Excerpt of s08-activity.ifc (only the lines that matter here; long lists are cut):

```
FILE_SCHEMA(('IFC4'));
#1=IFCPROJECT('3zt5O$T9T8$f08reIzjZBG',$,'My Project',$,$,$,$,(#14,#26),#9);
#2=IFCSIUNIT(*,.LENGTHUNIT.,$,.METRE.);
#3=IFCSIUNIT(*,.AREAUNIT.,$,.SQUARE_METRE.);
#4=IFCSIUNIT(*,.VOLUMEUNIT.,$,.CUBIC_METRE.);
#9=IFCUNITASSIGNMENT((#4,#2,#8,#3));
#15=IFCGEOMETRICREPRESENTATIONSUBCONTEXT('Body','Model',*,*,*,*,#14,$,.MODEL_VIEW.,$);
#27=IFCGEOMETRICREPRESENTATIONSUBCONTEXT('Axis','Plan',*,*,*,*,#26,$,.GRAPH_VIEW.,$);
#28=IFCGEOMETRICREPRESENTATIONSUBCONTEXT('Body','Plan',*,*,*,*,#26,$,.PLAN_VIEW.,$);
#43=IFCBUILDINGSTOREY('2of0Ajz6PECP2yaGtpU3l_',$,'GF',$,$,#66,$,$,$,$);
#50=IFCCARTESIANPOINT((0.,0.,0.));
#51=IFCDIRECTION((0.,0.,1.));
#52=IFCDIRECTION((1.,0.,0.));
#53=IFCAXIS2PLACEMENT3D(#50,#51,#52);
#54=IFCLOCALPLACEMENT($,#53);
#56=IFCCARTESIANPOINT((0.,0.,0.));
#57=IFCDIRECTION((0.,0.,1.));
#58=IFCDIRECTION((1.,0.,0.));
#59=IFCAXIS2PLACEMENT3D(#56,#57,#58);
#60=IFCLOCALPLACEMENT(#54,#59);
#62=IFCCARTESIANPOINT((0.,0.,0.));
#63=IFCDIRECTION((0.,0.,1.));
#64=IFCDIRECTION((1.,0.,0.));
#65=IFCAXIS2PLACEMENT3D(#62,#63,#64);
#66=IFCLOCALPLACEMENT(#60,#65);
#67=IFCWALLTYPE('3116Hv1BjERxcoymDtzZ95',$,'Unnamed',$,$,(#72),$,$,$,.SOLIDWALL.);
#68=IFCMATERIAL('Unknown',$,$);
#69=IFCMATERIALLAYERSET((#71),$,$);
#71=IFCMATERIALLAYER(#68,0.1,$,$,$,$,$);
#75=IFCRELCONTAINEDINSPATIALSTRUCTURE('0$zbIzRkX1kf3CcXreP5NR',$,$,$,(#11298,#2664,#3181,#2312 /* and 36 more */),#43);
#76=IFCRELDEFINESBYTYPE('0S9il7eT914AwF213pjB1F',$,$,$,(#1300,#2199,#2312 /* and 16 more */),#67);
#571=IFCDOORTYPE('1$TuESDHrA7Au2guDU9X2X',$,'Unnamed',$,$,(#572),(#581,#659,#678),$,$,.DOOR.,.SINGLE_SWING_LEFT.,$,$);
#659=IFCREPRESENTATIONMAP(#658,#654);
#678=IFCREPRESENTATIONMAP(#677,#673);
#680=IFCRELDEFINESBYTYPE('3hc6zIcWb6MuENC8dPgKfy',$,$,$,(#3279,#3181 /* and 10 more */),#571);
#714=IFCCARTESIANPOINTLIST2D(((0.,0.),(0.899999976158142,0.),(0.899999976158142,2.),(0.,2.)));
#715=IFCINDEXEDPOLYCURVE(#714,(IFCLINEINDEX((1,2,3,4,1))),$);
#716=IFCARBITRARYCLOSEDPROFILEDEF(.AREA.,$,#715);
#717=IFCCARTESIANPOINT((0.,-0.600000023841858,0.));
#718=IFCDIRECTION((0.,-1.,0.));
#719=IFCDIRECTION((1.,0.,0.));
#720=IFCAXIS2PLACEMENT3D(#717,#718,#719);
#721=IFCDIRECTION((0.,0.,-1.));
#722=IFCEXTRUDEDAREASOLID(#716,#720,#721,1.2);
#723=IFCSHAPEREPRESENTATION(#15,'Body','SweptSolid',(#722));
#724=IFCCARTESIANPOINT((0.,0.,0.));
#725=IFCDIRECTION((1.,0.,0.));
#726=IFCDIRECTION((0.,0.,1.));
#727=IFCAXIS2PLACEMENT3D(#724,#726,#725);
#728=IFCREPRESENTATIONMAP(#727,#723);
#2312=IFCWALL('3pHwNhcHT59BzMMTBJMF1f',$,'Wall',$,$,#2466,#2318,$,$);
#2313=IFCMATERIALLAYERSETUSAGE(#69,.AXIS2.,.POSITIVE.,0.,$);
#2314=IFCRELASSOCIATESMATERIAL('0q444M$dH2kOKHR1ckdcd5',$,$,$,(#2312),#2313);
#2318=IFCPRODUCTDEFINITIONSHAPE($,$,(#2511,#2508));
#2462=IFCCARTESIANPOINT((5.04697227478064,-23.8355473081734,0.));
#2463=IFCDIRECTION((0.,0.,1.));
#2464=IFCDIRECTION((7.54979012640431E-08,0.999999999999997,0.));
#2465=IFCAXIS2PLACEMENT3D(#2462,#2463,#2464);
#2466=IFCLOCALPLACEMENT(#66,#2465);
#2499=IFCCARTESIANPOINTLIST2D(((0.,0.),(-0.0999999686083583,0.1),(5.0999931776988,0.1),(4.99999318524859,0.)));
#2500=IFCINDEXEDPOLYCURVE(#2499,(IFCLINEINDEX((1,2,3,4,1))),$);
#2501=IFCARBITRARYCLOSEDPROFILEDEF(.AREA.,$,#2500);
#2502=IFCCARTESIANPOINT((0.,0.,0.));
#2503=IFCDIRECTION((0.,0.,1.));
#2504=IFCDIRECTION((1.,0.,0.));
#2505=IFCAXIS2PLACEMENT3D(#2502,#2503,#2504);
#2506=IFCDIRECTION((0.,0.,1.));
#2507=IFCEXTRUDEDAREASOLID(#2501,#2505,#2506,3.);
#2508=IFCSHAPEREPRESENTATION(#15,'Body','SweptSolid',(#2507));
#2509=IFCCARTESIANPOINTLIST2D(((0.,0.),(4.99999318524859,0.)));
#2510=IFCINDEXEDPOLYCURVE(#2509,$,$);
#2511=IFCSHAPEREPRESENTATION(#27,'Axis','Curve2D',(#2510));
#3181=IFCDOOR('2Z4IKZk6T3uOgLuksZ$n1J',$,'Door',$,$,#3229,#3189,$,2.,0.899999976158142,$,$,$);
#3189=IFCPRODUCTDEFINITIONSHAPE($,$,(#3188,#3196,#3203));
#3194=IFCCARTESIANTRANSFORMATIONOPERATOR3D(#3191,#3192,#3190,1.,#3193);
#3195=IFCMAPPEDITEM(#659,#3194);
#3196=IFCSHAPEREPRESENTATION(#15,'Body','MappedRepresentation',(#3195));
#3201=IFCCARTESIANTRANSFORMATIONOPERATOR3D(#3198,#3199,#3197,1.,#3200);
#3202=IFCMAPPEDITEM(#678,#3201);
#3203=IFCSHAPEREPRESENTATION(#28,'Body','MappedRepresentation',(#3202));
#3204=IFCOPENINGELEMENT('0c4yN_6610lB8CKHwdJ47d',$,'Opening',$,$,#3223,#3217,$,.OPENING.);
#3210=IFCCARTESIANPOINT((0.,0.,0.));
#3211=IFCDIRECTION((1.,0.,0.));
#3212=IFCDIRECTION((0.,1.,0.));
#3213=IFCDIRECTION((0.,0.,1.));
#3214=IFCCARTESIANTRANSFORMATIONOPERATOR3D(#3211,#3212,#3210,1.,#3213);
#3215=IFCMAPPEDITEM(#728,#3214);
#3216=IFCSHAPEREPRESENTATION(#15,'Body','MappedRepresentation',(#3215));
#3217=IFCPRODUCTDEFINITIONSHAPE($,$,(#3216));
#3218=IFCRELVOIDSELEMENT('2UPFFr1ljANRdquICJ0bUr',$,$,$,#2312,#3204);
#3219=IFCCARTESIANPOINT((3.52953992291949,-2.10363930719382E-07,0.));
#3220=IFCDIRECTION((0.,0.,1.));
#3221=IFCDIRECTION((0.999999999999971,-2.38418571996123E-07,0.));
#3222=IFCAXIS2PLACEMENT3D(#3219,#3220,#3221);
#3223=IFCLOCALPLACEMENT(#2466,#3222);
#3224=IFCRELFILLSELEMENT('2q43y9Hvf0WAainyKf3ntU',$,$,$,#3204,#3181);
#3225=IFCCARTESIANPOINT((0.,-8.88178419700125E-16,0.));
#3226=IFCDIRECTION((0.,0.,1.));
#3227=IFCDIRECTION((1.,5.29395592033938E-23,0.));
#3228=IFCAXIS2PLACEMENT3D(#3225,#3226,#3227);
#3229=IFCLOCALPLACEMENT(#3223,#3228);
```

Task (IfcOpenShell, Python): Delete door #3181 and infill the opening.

```python
import ifcopenshell
import ifcopenshell.api.feature
import ifcopenshell.api.root
import ifcopenshell.geom
import ifcopenshell.util.shape

model = ifcopenshell.open("s08-activity.ifc")
settings = ifcopenshell.geom.settings()


def volume(element):
    """Net volume in cubic metres, openings subtracted."""
    shape = ifcopenshell.geom.create_shape(settings, element)
    return ifcopenshell.util.shape.get_volume(shape.geometry)


door = model.by_id(3181)
opening = door.FillsVoids[0].RelatingOpeningElement
wall = opening.VoidsElements[0].RelatingBuildingElement
before = volume(wall)

ifcopenshell.api.root.remove_product(model, product=door)
ifcopenshell.api.feature.remove_feature(model, feature=opening)

after = volume(wall)

print(f"wall volume {before:.3f} -> {after:.3f} m3")

model.write("s08-activity_v2.ifc")
```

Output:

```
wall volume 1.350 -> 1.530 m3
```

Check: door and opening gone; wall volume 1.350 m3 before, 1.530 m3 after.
